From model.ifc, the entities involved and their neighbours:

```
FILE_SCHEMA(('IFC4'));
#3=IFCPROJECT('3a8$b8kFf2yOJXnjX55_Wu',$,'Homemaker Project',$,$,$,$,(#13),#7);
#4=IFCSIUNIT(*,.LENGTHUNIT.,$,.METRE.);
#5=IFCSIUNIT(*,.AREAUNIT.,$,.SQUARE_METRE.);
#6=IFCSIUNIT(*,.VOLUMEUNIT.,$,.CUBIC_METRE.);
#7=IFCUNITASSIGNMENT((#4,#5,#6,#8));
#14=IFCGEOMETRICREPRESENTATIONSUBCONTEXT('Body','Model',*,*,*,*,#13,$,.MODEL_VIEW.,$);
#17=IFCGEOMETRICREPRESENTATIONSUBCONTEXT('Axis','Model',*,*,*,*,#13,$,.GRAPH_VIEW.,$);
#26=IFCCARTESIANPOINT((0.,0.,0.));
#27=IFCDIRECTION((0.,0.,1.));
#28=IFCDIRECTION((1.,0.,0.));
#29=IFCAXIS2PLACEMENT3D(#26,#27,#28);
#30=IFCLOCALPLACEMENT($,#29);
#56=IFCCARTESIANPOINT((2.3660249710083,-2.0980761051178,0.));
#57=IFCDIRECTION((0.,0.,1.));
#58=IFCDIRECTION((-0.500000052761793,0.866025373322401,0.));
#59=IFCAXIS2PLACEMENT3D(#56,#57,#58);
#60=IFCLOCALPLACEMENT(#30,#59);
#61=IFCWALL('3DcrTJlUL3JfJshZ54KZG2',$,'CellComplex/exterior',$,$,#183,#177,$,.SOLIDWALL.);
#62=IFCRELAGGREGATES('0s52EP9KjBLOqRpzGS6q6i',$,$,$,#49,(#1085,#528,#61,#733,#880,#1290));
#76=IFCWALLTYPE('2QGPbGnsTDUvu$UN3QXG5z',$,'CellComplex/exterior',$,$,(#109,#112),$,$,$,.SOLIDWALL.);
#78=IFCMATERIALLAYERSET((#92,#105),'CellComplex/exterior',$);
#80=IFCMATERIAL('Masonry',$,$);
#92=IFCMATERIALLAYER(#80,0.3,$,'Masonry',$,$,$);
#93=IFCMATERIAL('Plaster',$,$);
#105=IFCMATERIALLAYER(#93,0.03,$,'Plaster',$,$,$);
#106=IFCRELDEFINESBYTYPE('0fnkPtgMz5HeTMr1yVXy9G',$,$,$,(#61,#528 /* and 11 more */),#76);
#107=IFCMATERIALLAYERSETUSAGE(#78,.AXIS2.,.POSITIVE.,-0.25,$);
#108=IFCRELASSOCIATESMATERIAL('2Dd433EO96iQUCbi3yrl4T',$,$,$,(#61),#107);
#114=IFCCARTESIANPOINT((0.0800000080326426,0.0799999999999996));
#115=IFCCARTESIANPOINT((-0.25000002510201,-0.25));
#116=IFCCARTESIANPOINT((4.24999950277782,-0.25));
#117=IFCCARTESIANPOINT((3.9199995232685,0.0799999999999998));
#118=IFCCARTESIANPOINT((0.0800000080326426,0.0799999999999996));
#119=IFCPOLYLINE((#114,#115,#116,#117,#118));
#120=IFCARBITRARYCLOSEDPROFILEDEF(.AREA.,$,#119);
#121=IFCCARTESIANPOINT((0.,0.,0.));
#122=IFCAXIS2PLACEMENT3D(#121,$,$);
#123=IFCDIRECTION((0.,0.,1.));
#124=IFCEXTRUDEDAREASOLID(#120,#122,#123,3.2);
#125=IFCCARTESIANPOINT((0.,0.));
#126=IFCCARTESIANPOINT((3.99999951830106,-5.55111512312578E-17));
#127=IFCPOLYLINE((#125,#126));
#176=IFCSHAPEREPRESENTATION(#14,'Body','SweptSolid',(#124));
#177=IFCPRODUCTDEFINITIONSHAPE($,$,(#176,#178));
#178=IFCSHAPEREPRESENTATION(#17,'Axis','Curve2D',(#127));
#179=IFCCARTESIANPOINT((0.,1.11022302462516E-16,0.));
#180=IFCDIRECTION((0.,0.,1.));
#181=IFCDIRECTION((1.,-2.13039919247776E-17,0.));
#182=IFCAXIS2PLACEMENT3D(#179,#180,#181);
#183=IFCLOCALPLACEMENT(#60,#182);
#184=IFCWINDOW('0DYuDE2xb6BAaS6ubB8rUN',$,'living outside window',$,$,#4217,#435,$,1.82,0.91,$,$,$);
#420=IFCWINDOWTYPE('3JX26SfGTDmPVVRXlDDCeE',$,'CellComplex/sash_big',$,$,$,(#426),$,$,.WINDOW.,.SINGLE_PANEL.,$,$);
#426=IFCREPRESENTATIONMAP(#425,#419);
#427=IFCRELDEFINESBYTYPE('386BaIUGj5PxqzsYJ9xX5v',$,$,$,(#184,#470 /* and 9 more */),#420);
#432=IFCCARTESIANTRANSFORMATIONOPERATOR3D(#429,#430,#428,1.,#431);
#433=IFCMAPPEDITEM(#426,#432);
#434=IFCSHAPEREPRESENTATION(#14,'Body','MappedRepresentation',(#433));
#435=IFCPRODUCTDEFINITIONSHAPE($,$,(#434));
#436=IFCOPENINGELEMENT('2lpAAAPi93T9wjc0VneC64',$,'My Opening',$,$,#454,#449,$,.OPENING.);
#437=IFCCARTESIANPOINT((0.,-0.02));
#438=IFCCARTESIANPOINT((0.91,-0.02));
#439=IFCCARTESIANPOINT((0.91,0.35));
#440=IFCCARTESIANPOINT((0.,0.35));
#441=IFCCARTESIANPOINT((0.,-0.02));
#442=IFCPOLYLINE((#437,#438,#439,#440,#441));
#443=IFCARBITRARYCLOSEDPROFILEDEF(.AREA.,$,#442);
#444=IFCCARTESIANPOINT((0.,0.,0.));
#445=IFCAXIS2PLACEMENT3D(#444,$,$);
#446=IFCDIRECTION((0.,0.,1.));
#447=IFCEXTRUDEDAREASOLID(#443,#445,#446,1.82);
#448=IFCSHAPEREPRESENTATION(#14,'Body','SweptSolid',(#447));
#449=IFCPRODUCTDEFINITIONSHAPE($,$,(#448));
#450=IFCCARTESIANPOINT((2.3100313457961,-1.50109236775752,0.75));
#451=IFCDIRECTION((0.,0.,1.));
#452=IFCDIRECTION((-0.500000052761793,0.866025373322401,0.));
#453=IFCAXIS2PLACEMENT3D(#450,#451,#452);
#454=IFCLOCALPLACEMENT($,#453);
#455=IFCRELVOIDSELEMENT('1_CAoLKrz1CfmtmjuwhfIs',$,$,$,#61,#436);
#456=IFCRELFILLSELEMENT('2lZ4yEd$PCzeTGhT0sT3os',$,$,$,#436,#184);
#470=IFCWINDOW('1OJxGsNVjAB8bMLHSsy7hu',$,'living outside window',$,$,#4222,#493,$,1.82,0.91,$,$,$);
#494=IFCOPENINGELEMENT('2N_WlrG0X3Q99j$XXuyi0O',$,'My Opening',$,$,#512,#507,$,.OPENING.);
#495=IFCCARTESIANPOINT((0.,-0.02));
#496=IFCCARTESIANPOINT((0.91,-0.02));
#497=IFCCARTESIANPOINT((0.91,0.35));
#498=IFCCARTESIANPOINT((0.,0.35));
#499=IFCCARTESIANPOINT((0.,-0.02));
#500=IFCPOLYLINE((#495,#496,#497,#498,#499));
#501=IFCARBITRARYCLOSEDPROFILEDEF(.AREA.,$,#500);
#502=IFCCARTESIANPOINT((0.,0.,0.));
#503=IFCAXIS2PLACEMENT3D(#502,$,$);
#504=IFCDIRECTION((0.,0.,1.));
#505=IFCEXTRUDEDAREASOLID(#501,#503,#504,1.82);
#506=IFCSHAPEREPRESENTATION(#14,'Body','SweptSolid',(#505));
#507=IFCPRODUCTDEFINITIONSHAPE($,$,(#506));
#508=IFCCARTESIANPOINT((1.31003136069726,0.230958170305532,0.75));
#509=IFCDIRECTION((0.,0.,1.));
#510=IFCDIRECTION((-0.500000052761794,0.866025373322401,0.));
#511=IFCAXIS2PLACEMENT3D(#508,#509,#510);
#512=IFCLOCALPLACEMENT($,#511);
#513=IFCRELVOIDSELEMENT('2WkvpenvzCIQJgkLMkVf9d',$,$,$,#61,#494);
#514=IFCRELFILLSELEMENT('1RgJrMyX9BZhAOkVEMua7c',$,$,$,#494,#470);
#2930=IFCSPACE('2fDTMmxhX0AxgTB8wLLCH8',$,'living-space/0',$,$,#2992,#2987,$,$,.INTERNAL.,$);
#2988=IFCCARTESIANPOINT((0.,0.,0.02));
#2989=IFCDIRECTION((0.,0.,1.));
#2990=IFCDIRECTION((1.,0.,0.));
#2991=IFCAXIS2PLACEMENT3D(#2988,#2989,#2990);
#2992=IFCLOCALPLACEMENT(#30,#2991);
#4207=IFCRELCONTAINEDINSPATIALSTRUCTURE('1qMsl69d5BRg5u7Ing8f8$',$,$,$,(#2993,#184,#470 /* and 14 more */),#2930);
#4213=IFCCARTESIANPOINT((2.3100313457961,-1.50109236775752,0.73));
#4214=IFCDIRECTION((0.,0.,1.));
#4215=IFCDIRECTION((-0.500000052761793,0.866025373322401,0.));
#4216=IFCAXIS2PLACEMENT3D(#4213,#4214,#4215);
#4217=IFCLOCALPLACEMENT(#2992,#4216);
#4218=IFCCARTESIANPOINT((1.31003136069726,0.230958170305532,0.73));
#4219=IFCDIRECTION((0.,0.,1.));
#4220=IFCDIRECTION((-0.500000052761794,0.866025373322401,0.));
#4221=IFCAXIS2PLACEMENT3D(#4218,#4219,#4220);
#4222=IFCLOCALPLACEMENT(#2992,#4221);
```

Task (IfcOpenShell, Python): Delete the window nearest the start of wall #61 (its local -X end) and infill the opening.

```python
import ifcopenshell
import ifcopenshell.api.feature
import ifcopenshell.api.root
import ifcopenshell.geom
import ifcopenshell.util.shape

model = ifcopenshell.open("model.ifc")
settings = ifcopenshell.geom.settings()


def volume(element):
    """Net volume in cubic metres, openings subtracted."""
    shape = ifcopenshell.geom.create_shape(settings, element)
    return ifcopenshell.util.shape.get_volume(shape.geometry)


window = model.by_guid("0DYuDE2xb6BAaS6ubB8rUN")
opening = window.FillsVoids[0].RelatingOpeningElement
wall = opening.VoidsElements[0].RelatingBuildingElement
before = volume(wall)

ifcopenshell.api.root.remove_product(model, product=window)
ifcopenshell.api.feature.remove_feature(model, feature=opening)

after = volume(wall)

print(f"wall volume {before:.3f} -> {after:.3f} m3")

model.write("model_edited.ifc")
```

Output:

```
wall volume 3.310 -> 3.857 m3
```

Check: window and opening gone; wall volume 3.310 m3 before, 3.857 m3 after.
